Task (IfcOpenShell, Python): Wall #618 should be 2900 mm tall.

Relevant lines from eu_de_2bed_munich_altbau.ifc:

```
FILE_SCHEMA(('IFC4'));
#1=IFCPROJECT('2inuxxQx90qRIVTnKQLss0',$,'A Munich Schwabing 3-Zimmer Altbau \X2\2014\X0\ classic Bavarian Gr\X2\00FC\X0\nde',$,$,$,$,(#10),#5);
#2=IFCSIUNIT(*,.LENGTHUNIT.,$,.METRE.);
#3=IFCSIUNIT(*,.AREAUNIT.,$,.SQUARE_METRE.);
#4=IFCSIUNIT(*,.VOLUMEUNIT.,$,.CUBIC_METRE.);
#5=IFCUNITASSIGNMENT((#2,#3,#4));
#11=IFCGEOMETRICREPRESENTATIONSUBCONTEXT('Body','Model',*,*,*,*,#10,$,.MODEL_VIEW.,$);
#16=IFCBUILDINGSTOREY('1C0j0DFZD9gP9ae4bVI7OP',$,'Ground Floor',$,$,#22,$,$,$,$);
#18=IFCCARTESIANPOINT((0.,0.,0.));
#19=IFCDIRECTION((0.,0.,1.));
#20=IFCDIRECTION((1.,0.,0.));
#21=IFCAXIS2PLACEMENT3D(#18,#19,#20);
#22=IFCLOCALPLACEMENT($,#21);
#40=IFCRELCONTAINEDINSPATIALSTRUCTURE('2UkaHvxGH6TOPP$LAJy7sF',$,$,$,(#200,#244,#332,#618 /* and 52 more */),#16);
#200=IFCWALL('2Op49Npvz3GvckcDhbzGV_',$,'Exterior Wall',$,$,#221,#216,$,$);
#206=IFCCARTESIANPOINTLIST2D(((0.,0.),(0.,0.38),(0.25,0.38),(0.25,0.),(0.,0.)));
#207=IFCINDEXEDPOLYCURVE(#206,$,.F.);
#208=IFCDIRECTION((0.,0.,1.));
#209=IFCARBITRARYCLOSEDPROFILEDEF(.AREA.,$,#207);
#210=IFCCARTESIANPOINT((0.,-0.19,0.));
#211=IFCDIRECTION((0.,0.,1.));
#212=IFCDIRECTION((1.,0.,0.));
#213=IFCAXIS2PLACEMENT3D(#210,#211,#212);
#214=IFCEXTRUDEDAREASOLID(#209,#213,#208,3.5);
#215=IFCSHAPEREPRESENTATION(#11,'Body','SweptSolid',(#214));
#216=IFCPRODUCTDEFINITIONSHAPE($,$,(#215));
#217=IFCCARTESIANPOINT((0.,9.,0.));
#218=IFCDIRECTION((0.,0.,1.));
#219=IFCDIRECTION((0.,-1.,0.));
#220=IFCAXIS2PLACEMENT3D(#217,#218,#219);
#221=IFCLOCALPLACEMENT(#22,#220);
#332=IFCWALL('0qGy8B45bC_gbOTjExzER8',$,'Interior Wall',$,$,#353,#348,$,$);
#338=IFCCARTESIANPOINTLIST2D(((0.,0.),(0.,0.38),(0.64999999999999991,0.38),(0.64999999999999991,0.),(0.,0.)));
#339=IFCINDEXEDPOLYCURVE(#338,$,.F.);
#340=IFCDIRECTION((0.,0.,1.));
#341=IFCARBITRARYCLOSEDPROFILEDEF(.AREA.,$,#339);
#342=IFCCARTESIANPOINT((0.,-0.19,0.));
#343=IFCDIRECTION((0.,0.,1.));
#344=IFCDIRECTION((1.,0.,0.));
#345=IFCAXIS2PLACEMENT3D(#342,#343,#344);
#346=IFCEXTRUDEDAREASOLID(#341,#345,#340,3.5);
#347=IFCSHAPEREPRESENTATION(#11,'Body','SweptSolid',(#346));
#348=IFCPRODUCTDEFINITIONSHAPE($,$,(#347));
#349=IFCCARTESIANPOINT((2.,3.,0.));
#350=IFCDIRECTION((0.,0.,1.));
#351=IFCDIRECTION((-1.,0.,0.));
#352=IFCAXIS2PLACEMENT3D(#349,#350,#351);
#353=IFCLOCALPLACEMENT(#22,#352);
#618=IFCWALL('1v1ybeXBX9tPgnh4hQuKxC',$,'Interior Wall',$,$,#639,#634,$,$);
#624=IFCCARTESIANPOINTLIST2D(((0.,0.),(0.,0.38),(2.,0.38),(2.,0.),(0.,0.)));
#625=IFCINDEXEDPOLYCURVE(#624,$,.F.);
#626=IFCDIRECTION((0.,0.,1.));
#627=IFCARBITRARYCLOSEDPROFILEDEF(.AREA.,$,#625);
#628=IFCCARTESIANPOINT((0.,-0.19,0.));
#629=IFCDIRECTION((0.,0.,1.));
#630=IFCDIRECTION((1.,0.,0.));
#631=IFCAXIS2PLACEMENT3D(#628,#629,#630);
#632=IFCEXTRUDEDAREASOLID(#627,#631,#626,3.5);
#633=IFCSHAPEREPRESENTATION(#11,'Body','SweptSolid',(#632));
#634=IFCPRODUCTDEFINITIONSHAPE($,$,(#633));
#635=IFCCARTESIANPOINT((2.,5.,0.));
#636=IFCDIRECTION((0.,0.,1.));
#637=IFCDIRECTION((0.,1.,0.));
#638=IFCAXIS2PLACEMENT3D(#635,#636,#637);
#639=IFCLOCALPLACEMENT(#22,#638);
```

```python
import ifcopenshell
import ifcopenshell.geom
import ifcopenshell.util.representation
import ifcopenshell.util.shape
import ifcopenshell.util.unit

model = ifcopenshell.open("eu_de_2bed_munich_altbau.ifc")
unit_scale = ifcopenshell.util.unit.calculate_unit_scale(model)
settings = ifcopenshell.geom.settings()


def volume(element):
    """Net volume in cubic metres, openings subtracted."""
    shape = ifcopenshell.geom.create_shape(settings, element)
    return ifcopenshell.util.shape.get_volume(shape.geometry)


wall = model.by_id(618)
before = volume(wall)

body = ifcopenshell.util.representation.get_representation(wall, "Model", "Body")
solid = body.Items[0]
old_height = solid.Depth
solid.Depth = 2.9 / unit_scale
after = volume(wall)

print(f"height {old_height:g} -> {solid.Depth:g}, volume {before:.3f} -> {after:.3f} m3")

model.write("eu_de_2bed_munich_altbau_edited.ifc")
```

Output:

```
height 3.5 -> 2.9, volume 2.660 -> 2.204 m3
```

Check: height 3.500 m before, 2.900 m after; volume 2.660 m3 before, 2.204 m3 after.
